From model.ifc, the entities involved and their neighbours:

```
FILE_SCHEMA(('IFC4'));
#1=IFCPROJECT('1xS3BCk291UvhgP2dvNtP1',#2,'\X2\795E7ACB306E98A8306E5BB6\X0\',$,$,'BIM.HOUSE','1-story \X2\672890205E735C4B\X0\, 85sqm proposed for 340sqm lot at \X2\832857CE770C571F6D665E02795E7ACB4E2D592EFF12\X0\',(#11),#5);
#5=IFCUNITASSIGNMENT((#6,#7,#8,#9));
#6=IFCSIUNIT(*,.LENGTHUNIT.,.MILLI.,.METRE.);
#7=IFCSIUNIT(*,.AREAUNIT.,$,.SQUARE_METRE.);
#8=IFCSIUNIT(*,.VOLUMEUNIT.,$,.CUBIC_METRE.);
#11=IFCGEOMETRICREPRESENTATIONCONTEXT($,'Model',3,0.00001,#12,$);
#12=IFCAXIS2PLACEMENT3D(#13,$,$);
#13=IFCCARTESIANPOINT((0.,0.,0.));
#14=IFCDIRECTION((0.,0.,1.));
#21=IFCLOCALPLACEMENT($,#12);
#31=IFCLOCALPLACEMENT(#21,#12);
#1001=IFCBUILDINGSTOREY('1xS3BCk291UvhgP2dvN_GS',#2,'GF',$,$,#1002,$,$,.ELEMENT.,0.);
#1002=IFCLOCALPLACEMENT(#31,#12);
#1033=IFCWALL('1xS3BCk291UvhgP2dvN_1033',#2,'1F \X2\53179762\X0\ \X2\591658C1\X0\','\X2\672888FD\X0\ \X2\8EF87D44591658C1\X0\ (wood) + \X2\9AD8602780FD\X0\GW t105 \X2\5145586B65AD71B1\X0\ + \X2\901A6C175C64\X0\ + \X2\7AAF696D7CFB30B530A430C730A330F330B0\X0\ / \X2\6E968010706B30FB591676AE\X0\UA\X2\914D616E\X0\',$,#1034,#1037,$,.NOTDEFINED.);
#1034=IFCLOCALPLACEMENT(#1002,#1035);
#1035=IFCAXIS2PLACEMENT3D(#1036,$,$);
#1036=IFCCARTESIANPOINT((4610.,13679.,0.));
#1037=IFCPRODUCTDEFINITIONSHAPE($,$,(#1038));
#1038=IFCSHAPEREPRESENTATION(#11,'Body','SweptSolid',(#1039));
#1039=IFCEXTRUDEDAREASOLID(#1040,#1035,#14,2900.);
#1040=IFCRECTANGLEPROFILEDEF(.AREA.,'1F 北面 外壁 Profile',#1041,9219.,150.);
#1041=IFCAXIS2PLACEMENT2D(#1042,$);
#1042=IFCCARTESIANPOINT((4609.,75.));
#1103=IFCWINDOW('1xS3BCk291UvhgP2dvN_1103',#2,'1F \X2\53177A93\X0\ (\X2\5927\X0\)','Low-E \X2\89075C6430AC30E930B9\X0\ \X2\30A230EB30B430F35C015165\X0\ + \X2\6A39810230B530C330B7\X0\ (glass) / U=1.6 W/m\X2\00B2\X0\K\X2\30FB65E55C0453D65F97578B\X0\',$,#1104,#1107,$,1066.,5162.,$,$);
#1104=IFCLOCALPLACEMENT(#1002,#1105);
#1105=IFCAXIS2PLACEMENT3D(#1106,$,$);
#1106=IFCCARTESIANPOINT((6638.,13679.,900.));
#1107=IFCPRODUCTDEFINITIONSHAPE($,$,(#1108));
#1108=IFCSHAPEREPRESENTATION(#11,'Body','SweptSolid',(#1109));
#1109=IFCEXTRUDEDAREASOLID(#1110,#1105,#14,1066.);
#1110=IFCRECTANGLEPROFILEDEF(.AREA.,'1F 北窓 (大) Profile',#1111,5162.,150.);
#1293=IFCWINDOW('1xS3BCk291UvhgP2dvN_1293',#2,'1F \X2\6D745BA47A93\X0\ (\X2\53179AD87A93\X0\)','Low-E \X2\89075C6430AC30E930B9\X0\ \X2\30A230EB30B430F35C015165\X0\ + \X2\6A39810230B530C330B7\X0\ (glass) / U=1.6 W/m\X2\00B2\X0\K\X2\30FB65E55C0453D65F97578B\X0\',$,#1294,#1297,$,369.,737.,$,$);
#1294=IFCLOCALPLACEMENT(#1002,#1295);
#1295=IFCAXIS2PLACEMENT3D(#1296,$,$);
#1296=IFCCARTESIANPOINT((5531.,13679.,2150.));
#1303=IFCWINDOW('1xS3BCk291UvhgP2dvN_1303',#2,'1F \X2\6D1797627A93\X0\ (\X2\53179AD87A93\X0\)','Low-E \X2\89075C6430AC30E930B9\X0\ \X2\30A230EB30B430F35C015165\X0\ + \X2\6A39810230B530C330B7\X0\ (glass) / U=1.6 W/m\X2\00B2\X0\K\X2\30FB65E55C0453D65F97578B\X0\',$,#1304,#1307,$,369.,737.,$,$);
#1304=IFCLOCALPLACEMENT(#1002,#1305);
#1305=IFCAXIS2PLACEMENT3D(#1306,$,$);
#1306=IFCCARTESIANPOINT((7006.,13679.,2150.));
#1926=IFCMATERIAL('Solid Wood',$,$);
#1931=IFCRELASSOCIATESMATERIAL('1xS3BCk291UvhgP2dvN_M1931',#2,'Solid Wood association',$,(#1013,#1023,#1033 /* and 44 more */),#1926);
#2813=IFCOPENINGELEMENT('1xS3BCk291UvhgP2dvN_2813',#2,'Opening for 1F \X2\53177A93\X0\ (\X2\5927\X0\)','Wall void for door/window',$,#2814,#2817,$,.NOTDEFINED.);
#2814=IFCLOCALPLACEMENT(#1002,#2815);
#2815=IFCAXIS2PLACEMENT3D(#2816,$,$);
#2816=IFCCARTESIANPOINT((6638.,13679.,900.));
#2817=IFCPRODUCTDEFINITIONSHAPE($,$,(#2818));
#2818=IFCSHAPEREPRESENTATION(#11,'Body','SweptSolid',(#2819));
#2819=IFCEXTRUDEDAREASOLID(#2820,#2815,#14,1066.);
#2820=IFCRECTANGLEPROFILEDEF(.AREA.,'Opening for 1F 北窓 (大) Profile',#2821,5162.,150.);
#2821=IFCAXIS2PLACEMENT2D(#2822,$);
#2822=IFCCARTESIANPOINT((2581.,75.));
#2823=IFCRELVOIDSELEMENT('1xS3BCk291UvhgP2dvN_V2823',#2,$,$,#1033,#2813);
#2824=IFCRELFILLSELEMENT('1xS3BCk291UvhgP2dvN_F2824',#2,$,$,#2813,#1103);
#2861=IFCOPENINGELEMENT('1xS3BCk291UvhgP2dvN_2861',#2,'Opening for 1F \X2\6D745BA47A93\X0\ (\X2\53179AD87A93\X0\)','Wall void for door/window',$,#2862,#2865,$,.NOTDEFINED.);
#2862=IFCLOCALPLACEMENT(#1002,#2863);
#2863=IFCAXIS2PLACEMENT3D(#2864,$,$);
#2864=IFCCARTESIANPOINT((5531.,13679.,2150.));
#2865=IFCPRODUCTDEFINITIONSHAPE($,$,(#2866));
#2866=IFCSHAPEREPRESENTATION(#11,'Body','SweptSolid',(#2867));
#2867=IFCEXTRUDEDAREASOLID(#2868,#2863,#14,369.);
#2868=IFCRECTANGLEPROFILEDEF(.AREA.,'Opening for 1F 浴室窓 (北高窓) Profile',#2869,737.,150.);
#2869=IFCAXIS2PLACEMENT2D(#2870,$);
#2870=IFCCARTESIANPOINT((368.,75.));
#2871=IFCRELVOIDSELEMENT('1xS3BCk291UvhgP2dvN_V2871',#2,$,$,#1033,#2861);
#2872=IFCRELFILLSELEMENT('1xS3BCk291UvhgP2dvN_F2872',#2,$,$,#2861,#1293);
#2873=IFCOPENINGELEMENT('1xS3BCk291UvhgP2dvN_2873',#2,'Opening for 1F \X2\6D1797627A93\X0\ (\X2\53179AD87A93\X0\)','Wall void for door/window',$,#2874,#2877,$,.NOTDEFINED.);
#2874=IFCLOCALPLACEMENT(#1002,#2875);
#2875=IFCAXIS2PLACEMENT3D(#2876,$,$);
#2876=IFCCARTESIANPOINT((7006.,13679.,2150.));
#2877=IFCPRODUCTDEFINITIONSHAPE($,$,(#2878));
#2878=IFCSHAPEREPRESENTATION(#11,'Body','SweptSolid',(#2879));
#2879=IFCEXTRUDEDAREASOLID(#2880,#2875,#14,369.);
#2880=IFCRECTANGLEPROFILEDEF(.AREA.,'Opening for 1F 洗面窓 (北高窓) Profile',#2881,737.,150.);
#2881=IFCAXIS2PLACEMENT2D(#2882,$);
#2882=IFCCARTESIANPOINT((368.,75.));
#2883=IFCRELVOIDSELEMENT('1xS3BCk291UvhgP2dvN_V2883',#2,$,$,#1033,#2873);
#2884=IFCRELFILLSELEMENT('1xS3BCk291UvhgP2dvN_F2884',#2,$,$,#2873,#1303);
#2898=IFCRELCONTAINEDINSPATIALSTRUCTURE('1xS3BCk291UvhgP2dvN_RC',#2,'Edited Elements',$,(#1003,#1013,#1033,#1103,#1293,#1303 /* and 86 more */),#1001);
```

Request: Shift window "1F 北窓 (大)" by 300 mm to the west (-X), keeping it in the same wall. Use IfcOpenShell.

```python
import ifcopenshell
import ifcopenshell.api.geometry
import ifcopenshell.util.placement
import ifcopenshell.util.unit

model = ifcopenshell.open("model.ifc")
unit_scale = ifcopenshell.util.unit.calculate_unit_scale(model)

window = model.by_guid("1xS3BCk291UvhgP2dvN_1103")
opening = window.FillsVoids[0].RelatingOpeningElement
wall = opening.VoidsElements[0].RelatingBuildingElement

wall_matrix = ifcopenshell.util.placement.get_local_placement(wall.ObjectPlacement)
shift = wall_matrix[:3, 0] * -0.3 / unit_scale
before = ifcopenshell.util.placement.get_local_placement(window.ObjectPlacement)[:3, 3].copy()

# The window is not placed relative to its opening, so move both.
for product in (opening, window):
    matrix = ifcopenshell.util.placement.get_local_placement(product.ObjectPlacement)
    matrix[:3, 3] += shift
    ifcopenshell.api.geometry.edit_object_placement(model, product=product, matrix=matrix, is_si=False)

after = ifcopenshell.util.placement.get_local_placement(window.ObjectPlacement)[:3, 3]
print("window moved by", (after - before).round(3) + 0.0)

model.write("model_updated.ifc")
```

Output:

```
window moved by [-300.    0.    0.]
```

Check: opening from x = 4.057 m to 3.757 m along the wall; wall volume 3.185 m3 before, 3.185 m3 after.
